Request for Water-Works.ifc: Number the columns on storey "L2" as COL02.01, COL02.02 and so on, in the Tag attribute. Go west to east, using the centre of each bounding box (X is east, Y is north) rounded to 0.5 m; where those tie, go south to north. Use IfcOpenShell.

First a look at what the model holds.

```python
import ifcopenshell
import ifcopenshell.util.element
import ifcopenshell.util.placement

model = ifcopenshell.open("Water-Works.ifc")
print(model.schema)
storey = next(s for s in model.by_type("IfcBuildingStorey") if s.Name == "L2")
columns = [e for e in ifcopenshell.util.element.get_decomposition(storey) if e.is_a("IfcColumn")]
for e in sorted(columns, key=lambda e: e.id()):
    origin = ifcopenshell.util.placement.get_local_placement(e.ObjectPlacement)[:3, 3]
    print(e.id(), e.Tag, e.Name, origin.round(2) + 0.0, sep=" | ")
```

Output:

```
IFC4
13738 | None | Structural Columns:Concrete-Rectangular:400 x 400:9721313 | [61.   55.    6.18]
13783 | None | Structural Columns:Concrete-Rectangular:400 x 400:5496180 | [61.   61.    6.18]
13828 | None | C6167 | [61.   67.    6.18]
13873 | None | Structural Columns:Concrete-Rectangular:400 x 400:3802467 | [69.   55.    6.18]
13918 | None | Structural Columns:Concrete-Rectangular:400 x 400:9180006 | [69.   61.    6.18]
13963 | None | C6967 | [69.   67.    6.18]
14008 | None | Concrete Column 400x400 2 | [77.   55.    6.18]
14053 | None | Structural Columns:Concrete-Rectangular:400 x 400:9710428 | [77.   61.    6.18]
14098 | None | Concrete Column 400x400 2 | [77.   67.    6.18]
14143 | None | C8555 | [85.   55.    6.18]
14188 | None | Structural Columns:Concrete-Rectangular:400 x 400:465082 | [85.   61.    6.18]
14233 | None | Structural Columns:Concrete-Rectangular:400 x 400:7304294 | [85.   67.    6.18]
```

```python
import ifcopenshell
import ifcopenshell.geom
import ifcopenshell.util.element
import ifcopenshell.util.shape

model = ifcopenshell.open("Water-Works.ifc")
settings = ifcopenshell.geom.settings()
settings.set("use-world-coords", True)


def centre(element):
    shape = ifcopenshell.geom.create_shape(settings, element)
    return ifcopenshell.util.shape.get_bbox_centroid(shape.geometry)


storey = next(s for s in model.by_type("IfcBuildingStorey") if s.Name == "L2")
columns = [e for e in ifcopenshell.util.element.get_decomposition(storey) if e.is_a("IfcColumn")]

# Insertion points can sit at a corner or the storey origin, so sort by the geometry (in metres).
centres = {e: centre(e) for e in columns}
columns.sort(key=lambda e: (round(centres[e][0] / 0.5), centres[e][1]))

for i, e in enumerate(columns, start=1):
    number = f"COL02.{i:02d}"
    e.Tag = number
    print(e.id(), number)

model.write("Water-Works_updated.ifc")
```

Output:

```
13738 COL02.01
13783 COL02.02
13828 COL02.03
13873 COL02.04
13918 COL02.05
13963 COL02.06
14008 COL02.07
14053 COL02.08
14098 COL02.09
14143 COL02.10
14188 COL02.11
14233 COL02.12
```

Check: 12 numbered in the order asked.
